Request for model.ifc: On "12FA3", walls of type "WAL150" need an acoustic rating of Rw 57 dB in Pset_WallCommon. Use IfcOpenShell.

First a look at what the model holds.

```python
import ifcopenshell
import ifcopenshell.util.element

model = ifcopenshell.open("model.ifc")
print(model.schema)
storey = next(s for s in model.by_type("IfcBuildingStorey") if s.Name == "12FA3")
walls = [e for e in ifcopenshell.util.element.get_decomposition(storey) if e.is_a("IfcWall")]
seen = {}
for e in walls:
    element_type = ifcopenshell.util.element.get_type(e)
    key = (element_type.Name if element_type != e and element_type else None, ifcopenshell.util.element.get_pset(e, "Pset_WallCommon", "AcousticRating"))
    seen[key] = seen.get(key, 0) + 1
for (name, value), count in sorted(seen.items(), key=str):
    print(count, "x", name, "|", value)
```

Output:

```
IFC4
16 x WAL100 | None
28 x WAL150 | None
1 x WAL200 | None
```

```python
import ifcopenshell
import ifcopenshell.api.pset
import ifcopenshell.util.element

model = ifcopenshell.open("model.ifc")

storey = next(s for s in model.by_type("IfcBuildingStorey") if s.Name == "12FA3")
walls = [e for e in ifcopenshell.util.element.get_decomposition(storey) if e.is_a("IfcWall")]

count = 0
for e in walls:
    element_type = ifcopenshell.util.element.get_type(e)
    if element_type in (None, e) or element_type.Name != "WAL150":
        continue
    # add_pset returns the element's existing set when there is one.
    pset = ifcopenshell.api.pset.add_pset(model, product=e, name="Pset_WallCommon")
    ifcopenshell.api.pset.edit_pset(model, pset=pset, properties={"AcousticRating": "Rw 57 dB"})
    count += 1

print(count, "walls updated")

model.write("model_v2.ifc")
```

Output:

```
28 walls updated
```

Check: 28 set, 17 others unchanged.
